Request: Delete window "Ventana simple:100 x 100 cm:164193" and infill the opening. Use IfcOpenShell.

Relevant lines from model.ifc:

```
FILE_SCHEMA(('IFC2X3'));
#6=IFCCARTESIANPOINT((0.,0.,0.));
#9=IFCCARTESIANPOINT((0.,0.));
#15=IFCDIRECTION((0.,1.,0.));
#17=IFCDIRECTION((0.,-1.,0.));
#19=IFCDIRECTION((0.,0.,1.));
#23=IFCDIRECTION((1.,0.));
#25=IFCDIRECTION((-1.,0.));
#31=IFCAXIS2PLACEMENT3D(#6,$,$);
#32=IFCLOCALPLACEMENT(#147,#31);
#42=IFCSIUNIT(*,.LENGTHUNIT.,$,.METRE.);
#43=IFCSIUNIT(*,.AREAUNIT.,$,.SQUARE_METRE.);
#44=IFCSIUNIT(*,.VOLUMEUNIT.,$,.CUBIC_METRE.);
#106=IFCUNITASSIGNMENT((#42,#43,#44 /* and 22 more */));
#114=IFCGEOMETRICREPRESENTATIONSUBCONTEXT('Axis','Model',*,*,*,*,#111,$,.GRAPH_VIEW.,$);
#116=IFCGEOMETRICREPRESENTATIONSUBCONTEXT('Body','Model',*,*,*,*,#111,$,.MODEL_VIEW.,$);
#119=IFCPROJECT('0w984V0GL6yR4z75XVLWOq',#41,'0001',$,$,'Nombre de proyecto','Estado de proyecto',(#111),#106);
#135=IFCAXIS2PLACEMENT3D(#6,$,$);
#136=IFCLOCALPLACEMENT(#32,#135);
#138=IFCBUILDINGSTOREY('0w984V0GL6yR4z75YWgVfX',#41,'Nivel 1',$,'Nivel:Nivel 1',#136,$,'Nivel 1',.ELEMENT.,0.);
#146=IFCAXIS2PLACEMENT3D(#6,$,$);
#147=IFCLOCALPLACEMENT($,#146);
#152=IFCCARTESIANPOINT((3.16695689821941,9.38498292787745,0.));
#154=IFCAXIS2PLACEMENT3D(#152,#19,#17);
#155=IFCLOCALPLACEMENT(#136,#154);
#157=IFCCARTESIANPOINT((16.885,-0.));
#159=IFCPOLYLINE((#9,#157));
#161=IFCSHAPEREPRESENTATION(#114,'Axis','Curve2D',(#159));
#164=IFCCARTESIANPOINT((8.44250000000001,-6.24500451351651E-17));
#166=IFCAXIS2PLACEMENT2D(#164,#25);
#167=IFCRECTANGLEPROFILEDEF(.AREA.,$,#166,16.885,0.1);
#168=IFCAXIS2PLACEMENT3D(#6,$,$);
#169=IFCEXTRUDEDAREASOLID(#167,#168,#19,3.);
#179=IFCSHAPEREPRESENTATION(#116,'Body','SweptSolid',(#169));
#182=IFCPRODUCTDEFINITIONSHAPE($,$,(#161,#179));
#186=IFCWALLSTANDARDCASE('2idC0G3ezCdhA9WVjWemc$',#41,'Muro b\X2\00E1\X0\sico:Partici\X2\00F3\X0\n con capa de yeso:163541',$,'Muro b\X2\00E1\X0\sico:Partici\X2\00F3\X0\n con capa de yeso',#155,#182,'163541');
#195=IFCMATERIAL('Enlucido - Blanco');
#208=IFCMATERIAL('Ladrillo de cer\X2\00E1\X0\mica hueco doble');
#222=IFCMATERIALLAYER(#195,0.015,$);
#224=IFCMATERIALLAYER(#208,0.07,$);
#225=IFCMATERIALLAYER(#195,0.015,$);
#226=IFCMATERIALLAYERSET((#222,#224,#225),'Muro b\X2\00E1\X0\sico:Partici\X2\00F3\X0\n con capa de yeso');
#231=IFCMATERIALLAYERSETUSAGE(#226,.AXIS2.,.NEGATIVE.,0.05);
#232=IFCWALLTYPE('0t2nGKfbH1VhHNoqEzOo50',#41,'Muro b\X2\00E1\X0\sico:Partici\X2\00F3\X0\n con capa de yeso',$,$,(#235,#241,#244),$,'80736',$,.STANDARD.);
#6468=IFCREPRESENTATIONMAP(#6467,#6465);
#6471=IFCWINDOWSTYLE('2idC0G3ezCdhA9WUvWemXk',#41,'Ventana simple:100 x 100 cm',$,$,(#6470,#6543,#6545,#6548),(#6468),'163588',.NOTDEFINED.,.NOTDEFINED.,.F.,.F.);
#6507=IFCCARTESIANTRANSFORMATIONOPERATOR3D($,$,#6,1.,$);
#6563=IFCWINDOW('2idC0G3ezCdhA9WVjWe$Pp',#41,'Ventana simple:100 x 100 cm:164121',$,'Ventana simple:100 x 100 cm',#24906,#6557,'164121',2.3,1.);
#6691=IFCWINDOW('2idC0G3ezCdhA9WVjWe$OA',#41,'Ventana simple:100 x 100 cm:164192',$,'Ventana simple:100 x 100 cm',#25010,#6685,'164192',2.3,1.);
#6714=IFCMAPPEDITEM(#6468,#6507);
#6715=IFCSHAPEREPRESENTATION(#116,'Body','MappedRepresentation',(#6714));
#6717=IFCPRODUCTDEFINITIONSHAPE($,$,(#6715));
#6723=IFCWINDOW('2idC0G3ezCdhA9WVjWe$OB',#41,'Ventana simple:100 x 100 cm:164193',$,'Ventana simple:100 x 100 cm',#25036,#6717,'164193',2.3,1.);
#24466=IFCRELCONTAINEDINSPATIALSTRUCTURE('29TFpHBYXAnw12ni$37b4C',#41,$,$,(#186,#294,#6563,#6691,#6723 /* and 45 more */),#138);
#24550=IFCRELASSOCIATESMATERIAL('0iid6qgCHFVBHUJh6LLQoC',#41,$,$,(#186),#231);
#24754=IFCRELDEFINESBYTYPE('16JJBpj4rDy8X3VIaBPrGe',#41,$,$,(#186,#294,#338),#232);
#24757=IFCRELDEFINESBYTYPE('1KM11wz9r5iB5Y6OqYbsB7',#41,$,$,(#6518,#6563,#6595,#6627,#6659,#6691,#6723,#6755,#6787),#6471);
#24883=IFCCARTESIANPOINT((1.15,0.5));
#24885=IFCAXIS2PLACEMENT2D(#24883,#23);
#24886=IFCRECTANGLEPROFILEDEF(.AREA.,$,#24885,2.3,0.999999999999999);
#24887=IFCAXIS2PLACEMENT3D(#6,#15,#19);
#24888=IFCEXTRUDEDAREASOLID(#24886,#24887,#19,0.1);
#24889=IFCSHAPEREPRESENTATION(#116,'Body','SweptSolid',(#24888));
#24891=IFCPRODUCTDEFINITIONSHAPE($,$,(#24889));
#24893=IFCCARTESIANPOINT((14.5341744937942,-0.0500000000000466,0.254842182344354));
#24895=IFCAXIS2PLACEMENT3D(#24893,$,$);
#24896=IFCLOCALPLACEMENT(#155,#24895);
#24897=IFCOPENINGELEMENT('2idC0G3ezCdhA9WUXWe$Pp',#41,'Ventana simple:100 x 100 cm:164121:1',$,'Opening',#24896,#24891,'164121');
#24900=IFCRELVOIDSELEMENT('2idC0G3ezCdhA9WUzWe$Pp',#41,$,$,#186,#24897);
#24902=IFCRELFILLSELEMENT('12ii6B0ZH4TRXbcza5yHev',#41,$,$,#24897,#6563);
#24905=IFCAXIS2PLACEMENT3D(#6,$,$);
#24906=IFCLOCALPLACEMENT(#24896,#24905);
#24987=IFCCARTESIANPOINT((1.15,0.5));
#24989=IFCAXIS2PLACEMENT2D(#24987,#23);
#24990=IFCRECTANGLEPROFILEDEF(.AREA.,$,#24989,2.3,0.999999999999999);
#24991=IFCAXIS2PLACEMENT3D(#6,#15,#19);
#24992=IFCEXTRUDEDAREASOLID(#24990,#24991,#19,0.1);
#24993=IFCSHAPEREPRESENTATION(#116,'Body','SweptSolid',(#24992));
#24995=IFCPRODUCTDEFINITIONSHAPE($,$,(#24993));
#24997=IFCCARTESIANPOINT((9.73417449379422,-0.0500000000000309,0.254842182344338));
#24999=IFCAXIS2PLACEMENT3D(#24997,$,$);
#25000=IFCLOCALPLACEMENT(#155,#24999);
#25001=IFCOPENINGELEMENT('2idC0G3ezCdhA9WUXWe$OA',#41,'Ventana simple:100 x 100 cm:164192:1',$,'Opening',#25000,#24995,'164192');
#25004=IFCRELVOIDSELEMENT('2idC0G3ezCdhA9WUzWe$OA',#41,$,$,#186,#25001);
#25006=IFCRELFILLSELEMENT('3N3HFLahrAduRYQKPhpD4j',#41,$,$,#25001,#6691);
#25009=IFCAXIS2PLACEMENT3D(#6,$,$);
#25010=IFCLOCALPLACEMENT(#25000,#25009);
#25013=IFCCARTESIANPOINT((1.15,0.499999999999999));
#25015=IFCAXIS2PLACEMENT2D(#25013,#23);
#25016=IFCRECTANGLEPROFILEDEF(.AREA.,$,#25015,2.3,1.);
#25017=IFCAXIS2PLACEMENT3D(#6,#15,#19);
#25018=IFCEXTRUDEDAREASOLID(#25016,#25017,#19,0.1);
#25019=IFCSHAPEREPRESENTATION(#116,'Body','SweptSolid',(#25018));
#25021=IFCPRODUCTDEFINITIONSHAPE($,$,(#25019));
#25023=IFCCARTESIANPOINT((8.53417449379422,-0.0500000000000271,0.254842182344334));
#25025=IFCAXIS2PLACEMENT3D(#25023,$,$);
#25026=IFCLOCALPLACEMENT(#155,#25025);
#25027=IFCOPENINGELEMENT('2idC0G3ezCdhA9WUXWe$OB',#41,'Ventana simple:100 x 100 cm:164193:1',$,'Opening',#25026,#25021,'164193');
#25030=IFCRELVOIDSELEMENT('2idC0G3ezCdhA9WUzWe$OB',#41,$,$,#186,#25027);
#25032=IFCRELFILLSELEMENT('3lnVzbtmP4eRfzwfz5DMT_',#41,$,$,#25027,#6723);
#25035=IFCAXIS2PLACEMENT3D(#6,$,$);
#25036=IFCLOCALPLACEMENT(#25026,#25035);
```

```python
import ifcopenshell
import ifcopenshell.api.feature
import ifcopenshell.api.root
import ifcopenshell.geom
import ifcopenshell.util.shape

model = ifcopenshell.open("model.ifc")
settings = ifcopenshell.geom.settings()


def volume(element):
    """Net volume in cubic metres, openings subtracted."""
    shape = ifcopenshell.geom.create_shape(settings, element)
    return ifcopenshell.util.shape.get_volume(shape.geometry)


window = model.by_guid("2idC0G3ezCdhA9WVjWe$OB")
opening = window.FillsVoids[0].RelatingOpeningElement
wall = opening.VoidsElements[0].RelatingBuildingElement
before = volume(wall)

ifcopenshell.api.root.remove_product(model, product=window)
ifcopenshell.api.feature.remove_feature(model, feature=opening)

after = volume(wall)

print(f"wall volume {before:.3f} -> {after:.3f} m3")

model.write("model_edited.ifc")
```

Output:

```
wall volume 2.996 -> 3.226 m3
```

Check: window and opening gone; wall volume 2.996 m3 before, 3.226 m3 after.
